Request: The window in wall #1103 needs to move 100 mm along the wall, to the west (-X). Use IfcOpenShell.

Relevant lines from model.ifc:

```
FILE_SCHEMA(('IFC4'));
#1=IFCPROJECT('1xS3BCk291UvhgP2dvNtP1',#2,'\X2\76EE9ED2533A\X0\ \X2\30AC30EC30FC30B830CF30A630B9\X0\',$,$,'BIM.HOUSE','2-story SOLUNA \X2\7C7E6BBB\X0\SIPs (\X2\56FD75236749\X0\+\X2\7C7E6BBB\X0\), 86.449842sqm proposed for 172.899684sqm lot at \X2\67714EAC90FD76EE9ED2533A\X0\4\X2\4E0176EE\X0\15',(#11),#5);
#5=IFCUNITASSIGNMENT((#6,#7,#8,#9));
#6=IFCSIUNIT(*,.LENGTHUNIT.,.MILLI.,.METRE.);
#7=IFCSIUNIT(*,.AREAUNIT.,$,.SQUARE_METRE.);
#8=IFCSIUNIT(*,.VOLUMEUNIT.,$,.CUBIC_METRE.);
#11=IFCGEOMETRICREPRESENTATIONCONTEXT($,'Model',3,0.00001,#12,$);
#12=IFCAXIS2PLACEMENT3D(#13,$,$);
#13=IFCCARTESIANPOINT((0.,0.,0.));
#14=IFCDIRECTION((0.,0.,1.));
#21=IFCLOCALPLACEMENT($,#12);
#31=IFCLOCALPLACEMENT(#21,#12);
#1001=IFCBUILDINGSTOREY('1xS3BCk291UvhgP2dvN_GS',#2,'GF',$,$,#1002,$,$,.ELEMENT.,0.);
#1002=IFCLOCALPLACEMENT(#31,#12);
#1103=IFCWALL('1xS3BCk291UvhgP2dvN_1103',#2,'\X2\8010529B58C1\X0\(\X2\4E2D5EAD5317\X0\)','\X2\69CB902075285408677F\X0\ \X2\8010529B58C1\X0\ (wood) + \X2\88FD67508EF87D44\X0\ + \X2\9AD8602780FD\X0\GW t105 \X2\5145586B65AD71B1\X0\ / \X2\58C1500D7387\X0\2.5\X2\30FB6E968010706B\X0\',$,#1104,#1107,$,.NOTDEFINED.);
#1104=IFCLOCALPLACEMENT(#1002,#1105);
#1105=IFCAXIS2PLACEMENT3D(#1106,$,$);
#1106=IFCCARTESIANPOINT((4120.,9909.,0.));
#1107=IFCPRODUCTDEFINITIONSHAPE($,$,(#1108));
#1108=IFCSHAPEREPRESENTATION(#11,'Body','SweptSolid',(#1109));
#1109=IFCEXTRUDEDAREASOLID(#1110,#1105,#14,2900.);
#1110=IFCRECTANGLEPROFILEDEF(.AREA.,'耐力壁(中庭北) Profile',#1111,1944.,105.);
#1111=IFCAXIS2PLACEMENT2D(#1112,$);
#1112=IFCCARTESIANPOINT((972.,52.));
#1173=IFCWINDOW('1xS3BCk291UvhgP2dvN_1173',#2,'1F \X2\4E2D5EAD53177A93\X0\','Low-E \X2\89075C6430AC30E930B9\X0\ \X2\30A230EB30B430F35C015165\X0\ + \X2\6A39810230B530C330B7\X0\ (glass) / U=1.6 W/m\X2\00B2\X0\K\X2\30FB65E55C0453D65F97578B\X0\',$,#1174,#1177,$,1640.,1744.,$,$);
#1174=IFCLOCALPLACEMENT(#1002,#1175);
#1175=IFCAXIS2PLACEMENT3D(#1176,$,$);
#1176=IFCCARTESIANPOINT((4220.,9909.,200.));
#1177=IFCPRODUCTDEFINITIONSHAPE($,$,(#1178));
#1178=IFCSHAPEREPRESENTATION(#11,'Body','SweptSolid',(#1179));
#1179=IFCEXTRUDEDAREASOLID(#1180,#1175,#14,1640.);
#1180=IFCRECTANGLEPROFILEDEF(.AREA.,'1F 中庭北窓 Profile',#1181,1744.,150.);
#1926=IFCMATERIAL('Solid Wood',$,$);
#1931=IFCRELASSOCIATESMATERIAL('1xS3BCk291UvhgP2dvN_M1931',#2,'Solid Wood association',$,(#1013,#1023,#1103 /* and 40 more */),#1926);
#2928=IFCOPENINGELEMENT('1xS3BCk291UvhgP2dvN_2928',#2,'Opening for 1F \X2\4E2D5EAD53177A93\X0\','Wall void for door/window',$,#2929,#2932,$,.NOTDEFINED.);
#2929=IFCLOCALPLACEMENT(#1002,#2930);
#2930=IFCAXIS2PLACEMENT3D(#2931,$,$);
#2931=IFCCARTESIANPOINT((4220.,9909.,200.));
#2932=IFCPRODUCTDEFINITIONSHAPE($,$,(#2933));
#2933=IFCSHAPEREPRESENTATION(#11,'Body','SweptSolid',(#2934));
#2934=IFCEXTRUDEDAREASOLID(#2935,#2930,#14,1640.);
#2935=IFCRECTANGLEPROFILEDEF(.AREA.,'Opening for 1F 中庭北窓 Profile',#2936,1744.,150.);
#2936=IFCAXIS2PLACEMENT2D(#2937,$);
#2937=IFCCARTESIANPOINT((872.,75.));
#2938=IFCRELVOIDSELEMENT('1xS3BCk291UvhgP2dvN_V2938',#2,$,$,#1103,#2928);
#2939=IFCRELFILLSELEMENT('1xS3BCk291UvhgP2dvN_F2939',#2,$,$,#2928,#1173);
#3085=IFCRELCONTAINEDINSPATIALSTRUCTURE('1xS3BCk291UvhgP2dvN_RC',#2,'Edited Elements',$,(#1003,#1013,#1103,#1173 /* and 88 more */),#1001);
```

```python
import ifcopenshell
import ifcopenshell.api.geometry
import ifcopenshell.util.placement
import ifcopenshell.util.unit

model = ifcopenshell.open("model.ifc")
unit_scale = ifcopenshell.util.unit.calculate_unit_scale(model)

window = model.by_guid("1xS3BCk291UvhgP2dvN_1173")
opening = window.FillsVoids[0].RelatingOpeningElement
wall = opening.VoidsElements[0].RelatingBuildingElement

wall_matrix = ifcopenshell.util.placement.get_local_placement(wall.ObjectPlacement)
shift = wall_matrix[:3, 0] * -0.1 / unit_scale
before = ifcopenshell.util.placement.get_local_placement(window.ObjectPlacement)[:3, 3].copy()

# The window is not placed relative to its opening, so move both.
for product in (opening, window):
    matrix = ifcopenshell.util.placement.get_local_placement(product.ObjectPlacement)
    matrix[:3, 3] += shift
    ifcopenshell.api.geometry.edit_object_placement(model, product=product, matrix=matrix, is_si=False)

after = ifcopenshell.util.placement.get_local_placement(window.ObjectPlacement)[:3, 3]
print("window moved by", (after - before).round(3) + 0.0)

model.write("model_updated.ifc")
```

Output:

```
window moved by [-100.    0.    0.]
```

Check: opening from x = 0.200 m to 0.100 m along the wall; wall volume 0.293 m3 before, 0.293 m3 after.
